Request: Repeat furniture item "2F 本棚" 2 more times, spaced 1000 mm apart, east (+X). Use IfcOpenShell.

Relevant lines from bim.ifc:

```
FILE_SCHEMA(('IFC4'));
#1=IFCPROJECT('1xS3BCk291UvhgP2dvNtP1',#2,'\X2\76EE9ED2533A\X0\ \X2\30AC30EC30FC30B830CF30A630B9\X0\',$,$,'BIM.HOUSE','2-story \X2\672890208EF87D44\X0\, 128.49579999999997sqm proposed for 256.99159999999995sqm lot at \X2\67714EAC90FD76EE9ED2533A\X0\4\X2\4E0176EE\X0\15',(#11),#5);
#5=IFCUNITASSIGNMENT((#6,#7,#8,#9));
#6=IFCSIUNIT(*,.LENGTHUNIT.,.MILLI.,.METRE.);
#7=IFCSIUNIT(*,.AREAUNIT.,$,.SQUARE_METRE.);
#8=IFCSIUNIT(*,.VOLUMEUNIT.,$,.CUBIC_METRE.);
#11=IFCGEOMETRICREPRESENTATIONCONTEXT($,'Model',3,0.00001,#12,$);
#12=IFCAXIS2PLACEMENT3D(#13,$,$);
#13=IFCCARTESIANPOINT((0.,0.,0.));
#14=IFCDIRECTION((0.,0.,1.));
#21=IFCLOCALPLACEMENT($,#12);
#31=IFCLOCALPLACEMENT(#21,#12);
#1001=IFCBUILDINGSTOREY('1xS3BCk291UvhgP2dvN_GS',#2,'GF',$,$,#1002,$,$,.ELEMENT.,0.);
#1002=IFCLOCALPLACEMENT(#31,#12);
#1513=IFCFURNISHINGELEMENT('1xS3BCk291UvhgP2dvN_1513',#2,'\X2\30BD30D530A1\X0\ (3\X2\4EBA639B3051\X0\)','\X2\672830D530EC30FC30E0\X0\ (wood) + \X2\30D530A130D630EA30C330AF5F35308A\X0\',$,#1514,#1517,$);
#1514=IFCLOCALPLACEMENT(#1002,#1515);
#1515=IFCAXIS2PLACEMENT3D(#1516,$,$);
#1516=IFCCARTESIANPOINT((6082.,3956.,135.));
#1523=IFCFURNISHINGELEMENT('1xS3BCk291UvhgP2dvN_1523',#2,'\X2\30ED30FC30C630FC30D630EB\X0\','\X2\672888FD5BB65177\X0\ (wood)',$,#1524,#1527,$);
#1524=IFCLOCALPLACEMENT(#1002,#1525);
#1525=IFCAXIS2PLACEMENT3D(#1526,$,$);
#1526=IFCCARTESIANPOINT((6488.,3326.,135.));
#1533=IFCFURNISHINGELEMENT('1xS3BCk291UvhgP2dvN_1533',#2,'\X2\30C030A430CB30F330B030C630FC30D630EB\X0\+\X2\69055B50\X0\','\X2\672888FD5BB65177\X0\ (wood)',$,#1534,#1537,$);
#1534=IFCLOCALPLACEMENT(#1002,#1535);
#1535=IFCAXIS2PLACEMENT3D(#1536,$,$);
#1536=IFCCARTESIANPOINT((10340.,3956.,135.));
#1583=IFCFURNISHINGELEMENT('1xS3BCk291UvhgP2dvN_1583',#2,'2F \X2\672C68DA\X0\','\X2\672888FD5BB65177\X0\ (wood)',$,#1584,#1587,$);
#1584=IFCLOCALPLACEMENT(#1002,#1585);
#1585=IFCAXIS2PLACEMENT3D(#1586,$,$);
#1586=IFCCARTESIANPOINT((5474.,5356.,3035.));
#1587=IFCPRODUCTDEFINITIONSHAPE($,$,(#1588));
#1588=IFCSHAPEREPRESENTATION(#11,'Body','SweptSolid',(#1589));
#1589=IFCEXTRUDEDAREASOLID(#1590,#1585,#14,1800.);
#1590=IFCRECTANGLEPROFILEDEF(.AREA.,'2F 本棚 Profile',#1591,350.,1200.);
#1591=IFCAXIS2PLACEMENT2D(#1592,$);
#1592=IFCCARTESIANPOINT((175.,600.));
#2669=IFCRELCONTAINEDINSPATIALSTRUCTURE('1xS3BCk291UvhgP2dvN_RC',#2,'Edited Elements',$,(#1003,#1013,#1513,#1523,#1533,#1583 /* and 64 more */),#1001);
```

```python
import numpy as np
import ifcopenshell
import ifcopenshell.api.geometry
import ifcopenshell.api.root
import ifcopenshell.util.element
import ifcopenshell.util.placement
import ifcopenshell.util.unit

model = ifcopenshell.open("bim.ifc")
unit_scale = ifcopenshell.util.unit.calculate_unit_scale(model)


def reuse_history(source, copy):
    """copy_class also copies each property set's owner history, people and application; keep the originals."""
    for rel in copy.IsDefinedBy:
        if rel.is_a("IfcRelDefinesByProperties") and (history := rel.RelatingPropertyDefinition.OwnerHistory):
            rel.RelatingPropertyDefinition.OwnerHistory = source.OwnerHistory
            ifcopenshell.util.element.remove_deep2(model, history)


source = model.by_guid("1xS3BCk291UvhgP2dvN_1583")
base = ifcopenshell.util.placement.get_local_placement(source.ObjectPlacement)
step = np.array([1.0, 0.0, 0.0]) * 1 / unit_scale

for i in range(1, 3):
    copy = ifcopenshell.api.root.copy_class(model, product=source)
    copy.Representation = ifcopenshell.util.element.copy_deep(
        model, source.Representation, exclude=["IfcGeometricRepresentationContext", "IfcRepresentationMap"]
    )
    reuse_history(source, copy)
    matrix = base.copy()
    matrix[:3, 3] += i * step
    print("added at", matrix[:3, 3].round(3) + 0.0)
    ifcopenshell.api.geometry.edit_object_placement(model, product=copy, matrix=matrix, is_si=False)

model.write("bim-out.ifc")
```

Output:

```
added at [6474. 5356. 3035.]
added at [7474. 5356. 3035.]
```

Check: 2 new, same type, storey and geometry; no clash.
